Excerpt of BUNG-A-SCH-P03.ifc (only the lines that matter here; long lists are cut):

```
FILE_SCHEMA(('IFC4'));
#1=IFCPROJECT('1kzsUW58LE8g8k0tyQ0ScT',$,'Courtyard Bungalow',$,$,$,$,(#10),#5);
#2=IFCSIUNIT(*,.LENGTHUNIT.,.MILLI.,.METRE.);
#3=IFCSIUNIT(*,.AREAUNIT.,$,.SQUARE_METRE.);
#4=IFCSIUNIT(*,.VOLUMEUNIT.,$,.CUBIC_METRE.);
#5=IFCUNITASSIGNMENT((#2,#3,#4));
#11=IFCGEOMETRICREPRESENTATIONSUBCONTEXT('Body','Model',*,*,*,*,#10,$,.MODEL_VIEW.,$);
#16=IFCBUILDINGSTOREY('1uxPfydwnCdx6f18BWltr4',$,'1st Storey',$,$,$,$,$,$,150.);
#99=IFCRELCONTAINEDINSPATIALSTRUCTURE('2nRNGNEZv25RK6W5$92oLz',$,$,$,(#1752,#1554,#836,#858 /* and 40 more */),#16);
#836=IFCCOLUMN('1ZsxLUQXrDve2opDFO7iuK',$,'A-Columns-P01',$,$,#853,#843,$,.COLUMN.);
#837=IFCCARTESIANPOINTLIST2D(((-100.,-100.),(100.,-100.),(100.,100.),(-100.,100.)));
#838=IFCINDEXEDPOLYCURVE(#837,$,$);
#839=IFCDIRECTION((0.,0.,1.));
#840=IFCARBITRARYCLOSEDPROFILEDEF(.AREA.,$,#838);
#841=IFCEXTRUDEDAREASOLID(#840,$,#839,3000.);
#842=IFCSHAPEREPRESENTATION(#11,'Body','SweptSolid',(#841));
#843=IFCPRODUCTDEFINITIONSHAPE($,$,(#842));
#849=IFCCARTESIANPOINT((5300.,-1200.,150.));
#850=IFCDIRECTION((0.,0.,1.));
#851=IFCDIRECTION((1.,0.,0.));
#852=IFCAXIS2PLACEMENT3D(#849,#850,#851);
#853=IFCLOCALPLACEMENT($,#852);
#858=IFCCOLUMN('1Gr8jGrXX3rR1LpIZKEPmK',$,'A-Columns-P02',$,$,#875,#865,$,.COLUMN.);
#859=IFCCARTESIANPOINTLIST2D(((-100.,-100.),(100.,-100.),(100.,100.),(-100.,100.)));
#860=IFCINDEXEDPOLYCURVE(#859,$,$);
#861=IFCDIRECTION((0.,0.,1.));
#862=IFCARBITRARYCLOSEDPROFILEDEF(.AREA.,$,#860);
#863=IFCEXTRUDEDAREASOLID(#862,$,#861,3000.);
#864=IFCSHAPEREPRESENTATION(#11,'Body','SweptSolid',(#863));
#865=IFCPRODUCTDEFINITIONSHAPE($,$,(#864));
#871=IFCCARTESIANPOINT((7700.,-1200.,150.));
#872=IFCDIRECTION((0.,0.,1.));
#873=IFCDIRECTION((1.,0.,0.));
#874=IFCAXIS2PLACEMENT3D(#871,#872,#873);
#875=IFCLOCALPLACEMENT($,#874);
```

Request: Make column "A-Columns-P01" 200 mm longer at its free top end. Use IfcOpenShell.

```python
import ifcopenshell
import ifcopenshell.util.representation
import ifcopenshell.util.unit

model = ifcopenshell.open("BUNG-A-SCH-P03.ifc")
unit_scale = ifcopenshell.util.unit.calculate_unit_scale(model)

member = model.by_guid("1ZsxLUQXrDve2opDFO7iuK")
change = 0.2 / unit_scale

# The extrusion runs towards the end named, so only its depth changes.
body = ifcopenshell.util.representation.get_representation(member, "Model", "Body")
solid = body.Items[0]
old_length = solid.Depth
solid.Depth += change

print(f"length {old_length:g} -> {solid.Depth:g}")

model.write("BUNG-A-SCH-P03_v2.ifc")
```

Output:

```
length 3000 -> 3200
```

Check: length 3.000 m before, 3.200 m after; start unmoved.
